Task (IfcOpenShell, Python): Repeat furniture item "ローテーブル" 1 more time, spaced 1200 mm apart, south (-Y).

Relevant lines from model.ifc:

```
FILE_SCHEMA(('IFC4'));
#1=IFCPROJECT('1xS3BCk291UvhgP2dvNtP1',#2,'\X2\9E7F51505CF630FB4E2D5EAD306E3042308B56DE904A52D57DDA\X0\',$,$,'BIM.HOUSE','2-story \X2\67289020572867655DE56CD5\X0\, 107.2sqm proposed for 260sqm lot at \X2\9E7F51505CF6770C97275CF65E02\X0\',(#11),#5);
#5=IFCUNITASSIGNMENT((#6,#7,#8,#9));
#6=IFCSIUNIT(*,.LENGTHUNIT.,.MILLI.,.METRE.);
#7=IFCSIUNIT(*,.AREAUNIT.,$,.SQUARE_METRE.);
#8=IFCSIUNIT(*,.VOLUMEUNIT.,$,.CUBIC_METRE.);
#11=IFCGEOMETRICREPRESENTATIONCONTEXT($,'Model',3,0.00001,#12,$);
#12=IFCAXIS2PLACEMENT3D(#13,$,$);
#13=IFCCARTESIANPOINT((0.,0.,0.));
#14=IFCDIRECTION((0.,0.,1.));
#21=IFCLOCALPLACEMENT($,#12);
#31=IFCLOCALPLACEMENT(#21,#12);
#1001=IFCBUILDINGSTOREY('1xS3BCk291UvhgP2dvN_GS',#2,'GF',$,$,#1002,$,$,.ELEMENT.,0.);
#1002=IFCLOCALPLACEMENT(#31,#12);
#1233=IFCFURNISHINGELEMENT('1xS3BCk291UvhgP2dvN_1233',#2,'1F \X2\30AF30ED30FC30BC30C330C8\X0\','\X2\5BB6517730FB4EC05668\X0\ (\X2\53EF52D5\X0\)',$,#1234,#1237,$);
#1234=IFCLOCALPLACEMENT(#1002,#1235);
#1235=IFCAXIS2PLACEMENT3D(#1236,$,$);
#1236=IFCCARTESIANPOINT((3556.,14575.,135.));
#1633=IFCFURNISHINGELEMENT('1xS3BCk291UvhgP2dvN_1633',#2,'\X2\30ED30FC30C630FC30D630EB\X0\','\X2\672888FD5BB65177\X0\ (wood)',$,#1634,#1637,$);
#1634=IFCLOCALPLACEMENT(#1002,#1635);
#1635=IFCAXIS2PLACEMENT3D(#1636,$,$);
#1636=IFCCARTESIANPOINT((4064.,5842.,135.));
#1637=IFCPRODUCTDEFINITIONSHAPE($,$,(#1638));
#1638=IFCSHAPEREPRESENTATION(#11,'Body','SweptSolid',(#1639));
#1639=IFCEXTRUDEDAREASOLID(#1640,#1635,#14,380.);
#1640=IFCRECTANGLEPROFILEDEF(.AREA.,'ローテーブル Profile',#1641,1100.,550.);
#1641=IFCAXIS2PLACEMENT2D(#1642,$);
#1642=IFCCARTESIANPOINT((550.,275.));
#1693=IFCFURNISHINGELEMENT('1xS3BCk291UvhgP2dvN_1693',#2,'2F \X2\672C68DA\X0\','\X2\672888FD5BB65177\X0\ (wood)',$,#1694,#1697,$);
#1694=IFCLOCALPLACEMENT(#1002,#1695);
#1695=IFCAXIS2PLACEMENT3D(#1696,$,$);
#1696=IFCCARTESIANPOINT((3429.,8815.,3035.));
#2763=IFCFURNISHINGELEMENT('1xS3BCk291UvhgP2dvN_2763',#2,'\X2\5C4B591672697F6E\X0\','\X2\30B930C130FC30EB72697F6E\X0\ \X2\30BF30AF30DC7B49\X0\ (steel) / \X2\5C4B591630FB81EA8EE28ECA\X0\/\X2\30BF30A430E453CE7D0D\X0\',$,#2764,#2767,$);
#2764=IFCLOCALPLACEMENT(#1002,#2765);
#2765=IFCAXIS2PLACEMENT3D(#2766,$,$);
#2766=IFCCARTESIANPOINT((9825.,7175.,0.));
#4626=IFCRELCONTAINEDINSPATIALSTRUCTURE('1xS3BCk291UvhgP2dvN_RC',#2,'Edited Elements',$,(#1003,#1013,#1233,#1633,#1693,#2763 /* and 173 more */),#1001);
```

```python
import numpy as np
import ifcopenshell
import ifcopenshell.api.geometry
import ifcopenshell.api.root
import ifcopenshell.util.element
import ifcopenshell.util.placement

model = ifcopenshell.open("model.ifc")


def reuse_history(source, copy):
    """copy_class also copies each property set's owner history, people and application; keep the originals."""
    for rel in copy.IsDefinedBy:
        if rel.is_a("IfcRelDefinesByProperties") and (history := rel.RelatingPropertyDefinition.OwnerHistory):
            rel.RelatingPropertyDefinition.OwnerHistory = source.OwnerHistory
            ifcopenshell.util.element.remove_deep2(model, history)


source = model.by_id(1633)
base = ifcopenshell.util.placement.get_local_placement(source.ObjectPlacement)
step = np.array([0.0, -1.0, 0.0]) * 1200.0

for i in range(1, 2):
    copy = ifcopenshell.api.root.copy_class(model, product=source)
    copy.Representation = ifcopenshell.util.element.copy_deep(
        model, source.Representation, exclude=["IfcGeometricRepresentationContext", "IfcRepresentationMap"]
    )
    reuse_history(source, copy)
    matrix = base.copy()
    matrix[:3, 3] += i * step
    print("added at", matrix[:3, 3].round(3) + 0.0)
    ifcopenshell.api.geometry.edit_object_placement(model, product=copy, matrix=matrix, is_si=False)

model.write("model_rev.ifc")
```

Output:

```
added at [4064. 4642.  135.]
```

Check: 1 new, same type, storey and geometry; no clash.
